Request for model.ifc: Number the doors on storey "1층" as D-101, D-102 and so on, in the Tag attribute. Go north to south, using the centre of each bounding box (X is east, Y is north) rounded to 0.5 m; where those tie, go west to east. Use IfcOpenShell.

First a look at what the model holds.

```python
import ifcopenshell
import ifcopenshell.util.element
import ifcopenshell.util.placement

model = ifcopenshell.open("model.ifc")
print(model.schema)
storey = next(s for s in model.by_type("IfcBuildingStorey") if s.Name == "1층")
doors = [e for e in ifcopenshell.util.element.get_decomposition(storey) if e.is_a("IfcDoor")]
for e in sorted(doors, key=lambda e: e.id()):
    origin = ifcopenshell.util.placement.get_local_placement(e.ObjectPlacement)[:3, 3]
    print(e.id(), e.Tag, e.Name, origin.round(2) + 0.0, sep=" | ")
```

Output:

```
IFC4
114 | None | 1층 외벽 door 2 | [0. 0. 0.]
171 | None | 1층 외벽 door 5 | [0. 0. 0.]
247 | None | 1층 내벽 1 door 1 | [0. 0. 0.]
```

```python
import ifcopenshell
import ifcopenshell.geom
import ifcopenshell.util.element
import ifcopenshell.util.shape

model = ifcopenshell.open("model.ifc")
settings = ifcopenshell.geom.settings()
settings.set("use-world-coords", True)


def centre(element):
    shape = ifcopenshell.geom.create_shape(settings, element)
    return ifcopenshell.util.shape.get_bbox_centroid(shape.geometry)


storey = next(s for s in model.by_type("IfcBuildingStorey") if s.Name == "1층")
doors = [e for e in ifcopenshell.util.element.get_decomposition(storey) if e.is_a("IfcDoor")]

# Insertion points can sit at a corner or the storey origin, so sort by the geometry (in metres).
centres = {e: centre(e) for e in doors}
doors.sort(key=lambda e: (-round(centres[e][1] / 0.5), centres[e][0]))

for i, e in enumerate(doors, start=1):
    number = f"D-1{i:02d}"
    e.Tag = number
    print(e.id(), number)

model.write("model_edited.ifc")
```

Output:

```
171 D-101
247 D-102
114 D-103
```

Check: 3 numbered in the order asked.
